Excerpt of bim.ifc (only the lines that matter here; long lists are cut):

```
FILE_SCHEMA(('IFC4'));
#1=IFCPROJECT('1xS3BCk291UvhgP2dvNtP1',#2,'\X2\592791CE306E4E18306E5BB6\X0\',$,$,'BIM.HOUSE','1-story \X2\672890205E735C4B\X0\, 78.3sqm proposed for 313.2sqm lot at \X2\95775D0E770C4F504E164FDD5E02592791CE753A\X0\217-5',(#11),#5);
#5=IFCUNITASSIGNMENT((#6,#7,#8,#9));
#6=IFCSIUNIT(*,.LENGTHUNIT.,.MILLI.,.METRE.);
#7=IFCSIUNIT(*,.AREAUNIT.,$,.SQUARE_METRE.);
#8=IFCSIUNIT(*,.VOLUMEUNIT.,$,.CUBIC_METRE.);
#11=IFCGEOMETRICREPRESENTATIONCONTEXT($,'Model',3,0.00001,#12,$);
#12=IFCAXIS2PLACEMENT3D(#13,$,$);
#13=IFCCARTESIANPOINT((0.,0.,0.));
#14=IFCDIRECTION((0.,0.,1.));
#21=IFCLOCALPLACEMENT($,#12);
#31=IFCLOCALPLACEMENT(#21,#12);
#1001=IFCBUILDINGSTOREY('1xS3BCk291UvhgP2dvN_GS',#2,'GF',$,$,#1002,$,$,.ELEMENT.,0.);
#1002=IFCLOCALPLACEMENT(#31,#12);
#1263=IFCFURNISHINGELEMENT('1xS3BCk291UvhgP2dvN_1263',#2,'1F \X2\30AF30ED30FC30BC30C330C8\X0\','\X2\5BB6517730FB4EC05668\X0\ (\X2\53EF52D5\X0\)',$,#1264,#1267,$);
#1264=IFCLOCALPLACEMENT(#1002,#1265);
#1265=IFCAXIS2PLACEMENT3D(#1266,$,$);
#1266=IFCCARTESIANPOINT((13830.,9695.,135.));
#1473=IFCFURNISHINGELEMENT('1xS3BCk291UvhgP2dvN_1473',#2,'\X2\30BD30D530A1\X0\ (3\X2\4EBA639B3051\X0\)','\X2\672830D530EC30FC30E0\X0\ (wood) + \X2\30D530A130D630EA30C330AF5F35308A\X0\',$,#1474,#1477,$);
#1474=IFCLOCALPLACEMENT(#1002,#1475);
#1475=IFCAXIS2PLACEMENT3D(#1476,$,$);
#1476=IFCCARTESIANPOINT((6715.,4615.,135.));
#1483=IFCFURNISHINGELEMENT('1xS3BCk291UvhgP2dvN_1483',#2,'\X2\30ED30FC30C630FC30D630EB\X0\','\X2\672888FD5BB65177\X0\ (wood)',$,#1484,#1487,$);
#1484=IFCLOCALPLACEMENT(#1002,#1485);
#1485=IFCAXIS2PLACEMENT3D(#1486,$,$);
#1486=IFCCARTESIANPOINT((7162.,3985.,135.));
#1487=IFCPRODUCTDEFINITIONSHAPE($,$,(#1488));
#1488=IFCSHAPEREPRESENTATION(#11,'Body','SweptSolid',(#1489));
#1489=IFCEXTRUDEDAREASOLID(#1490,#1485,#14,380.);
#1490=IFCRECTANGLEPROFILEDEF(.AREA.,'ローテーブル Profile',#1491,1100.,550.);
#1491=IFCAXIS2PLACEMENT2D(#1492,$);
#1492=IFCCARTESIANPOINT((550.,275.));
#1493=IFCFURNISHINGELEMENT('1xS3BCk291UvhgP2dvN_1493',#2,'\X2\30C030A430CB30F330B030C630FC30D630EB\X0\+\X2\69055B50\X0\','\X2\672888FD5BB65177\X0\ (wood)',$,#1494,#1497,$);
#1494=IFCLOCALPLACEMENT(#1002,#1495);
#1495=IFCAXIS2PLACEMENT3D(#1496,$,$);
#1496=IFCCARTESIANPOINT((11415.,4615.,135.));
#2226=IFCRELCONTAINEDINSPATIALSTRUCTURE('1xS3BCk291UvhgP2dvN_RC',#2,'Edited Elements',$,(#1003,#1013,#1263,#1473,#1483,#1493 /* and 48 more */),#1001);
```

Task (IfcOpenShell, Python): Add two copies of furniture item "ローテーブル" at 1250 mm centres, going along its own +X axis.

```python
import ifcopenshell
import ifcopenshell.api.geometry
import ifcopenshell.api.root
import ifcopenshell.util.element
import ifcopenshell.util.placement

model = ifcopenshell.open("bim.ifc")


def reuse_history(source, copy):
    """copy_class also copies each property set's owner history, people and application; keep the originals."""
    for rel in copy.IsDefinedBy:
        if rel.is_a("IfcRelDefinesByProperties") and (history := rel.RelatingPropertyDefinition.OwnerHistory):
            rel.RelatingPropertyDefinition.OwnerHistory = source.OwnerHistory
            ifcopenshell.util.element.remove_deep2(model, history)


source = model.by_guid("1xS3BCk291UvhgP2dvN_1483")
base = ifcopenshell.util.placement.get_local_placement(source.ObjectPlacement)
step = base[:3, 0] * 1250.0

for i in range(1, 3):
    copy = ifcopenshell.api.root.copy_class(model, product=source)
    copy.Representation = ifcopenshell.util.element.copy_deep(
        model, source.Representation, exclude=["IfcGeometricRepresentationContext", "IfcRepresentationMap"]
    )
    reuse_history(source, copy)
    matrix = base.copy()
    matrix[:3, 3] += i * step
    print("added at", matrix[:3, 3].round(3) + 0.0)
    ifcopenshell.api.geometry.edit_object_placement(model, product=copy, matrix=matrix, is_si=False)

model.write("bim_edited.ifc")
```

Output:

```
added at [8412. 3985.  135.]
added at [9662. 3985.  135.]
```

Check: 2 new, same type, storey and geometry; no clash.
